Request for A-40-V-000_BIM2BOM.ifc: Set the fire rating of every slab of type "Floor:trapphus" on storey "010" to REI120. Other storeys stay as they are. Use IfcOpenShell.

First a look at what the model holds.

```python
import ifcopenshell
import ifcopenshell.util.element

model = ifcopenshell.open("A-40-V-000_BIM2BOM.ifc")
print(model.schema)
storey = next(s for s in model.by_type("IfcBuildingStorey") if s.Name == "010")
slabs = [e for e in ifcopenshell.util.element.get_decomposition(storey) if e.is_a("IfcSlab")]
seen = {}
for e in slabs:
    element_type = ifcopenshell.util.element.get_type(e)
    key = (element_type.Name if element_type != e and element_type else None, ifcopenshell.util.element.get_pset(e, "Pset_SlabCommon", "FireRating"))
    seen[key] = seen.get(key, 0) + 1
for (name, value), count in sorted(seen.items(), key=str):
    print(count, "x", name, "|", value)
```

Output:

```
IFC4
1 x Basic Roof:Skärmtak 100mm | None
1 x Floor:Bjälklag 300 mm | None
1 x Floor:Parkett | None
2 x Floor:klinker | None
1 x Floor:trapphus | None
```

```python
import ifcopenshell
import ifcopenshell.api.pset
import ifcopenshell.util.element

model = ifcopenshell.open("A-40-V-000_BIM2BOM.ifc")

storey = next(s for s in model.by_type("IfcBuildingStorey") if s.Name == "010")
slabs = [e for e in ifcopenshell.util.element.get_decomposition(storey) if e.is_a("IfcSlab")]

count = 0
for e in slabs:
    element_type = ifcopenshell.util.element.get_type(e)
    if element_type in (None, e) or element_type.Name != "Floor:trapphus":
        continue
    # add_pset returns the element's existing set when there is one.
    pset = ifcopenshell.api.pset.add_pset(model, product=e, name="Pset_SlabCommon")
    ifcopenshell.api.pset.edit_pset(model, pset=pset, properties={"FireRating": "REI120"})
    count += 1

print(count, "slabs updated")

model.write("A-40-V-000_BIM2BOM_v2.ifc")
```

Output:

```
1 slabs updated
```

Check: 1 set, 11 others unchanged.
